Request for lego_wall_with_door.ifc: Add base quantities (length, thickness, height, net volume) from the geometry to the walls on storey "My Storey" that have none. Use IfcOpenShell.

First a look at what the model holds.

```python
import ifcopenshell
import ifcopenshell.util.element
import ifcopenshell.util.unit

model = ifcopenshell.open("lego_wall_with_door.ifc")
print(model.schema)
for unit_type in ("LENGTHUNIT", "AREAUNIT", "VOLUMEUNIT"):
    print(unit_type, ifcopenshell.util.unit.calculate_unit_scale(model, unit_type))
storey = next(s for s in model.by_type("IfcBuildingStorey") if s.Name == "My Storey")
walls = [e for e in ifcopenshell.util.element.get_decomposition(storey) if e.is_a("IfcWall")]
for e in sorted(walls, key=lambda e: e.id()):
    print(e.id(), e.is_a(), e.Name, list(ifcopenshell.util.element.get_psets(e, qtos_only=True)), sep=" | ")
```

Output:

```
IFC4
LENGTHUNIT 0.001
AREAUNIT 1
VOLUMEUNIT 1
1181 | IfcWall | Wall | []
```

```python
import ifcopenshell
import ifcopenshell.api.pset
import ifcopenshell.geom
import ifcopenshell.util.element
import ifcopenshell.util.shape
import ifcopenshell.util.unit

model = ifcopenshell.open("lego_wall_with_door.ifc")
unit_scale = ifcopenshell.util.unit.calculate_unit_scale(model)
volume_scale = ifcopenshell.util.unit.calculate_unit_scale(model, "VOLUMEUNIT")
settings = ifcopenshell.geom.settings()

storey = next(s for s in model.by_type("IfcBuildingStorey") if s.Name == "My Storey")
walls = [e for e in ifcopenshell.util.element.get_decomposition(storey) if e.is_a("IfcWall")]

for e in sorted(walls, key=lambda e: e.id()):
    if ifcopenshell.util.element.get_psets(e, qtos_only=True, should_inherit=False):
        continue
    # Geometry comes back in metres, in the element's own axes.
    shape = ifcopenshell.geom.create_shape(settings, e)
    values = {
        "Length": ifcopenshell.util.shape.get_x(shape.geometry) / unit_scale,
        "Width": ifcopenshell.util.shape.get_y(shape.geometry) / unit_scale,
        "Height": ifcopenshell.util.shape.get_z(shape.geometry) / unit_scale,
        "NetVolume": ifcopenshell.util.shape.get_volume(shape.geometry) / volume_scale,
    }
    qto = ifcopenshell.api.pset.add_qto(model, product=e, name="Qto_WallBaseQuantities")
    ifcopenshell.api.pset.edit_qto(model, qto=qto, properties=values)
    print(e.id(), {k: round(v, 3) for k, v in values.items()})

model.write("lego_wall_with_door-out.ifc")
```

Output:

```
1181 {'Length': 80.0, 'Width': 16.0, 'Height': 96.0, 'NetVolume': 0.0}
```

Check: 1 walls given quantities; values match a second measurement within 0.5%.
